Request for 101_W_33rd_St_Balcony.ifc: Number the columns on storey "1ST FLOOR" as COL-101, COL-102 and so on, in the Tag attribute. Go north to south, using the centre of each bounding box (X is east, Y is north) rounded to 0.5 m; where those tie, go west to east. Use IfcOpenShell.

First a look at what the model holds.

```python
import ifcopenshell
import ifcopenshell.util.element
import ifcopenshell.util.placement

model = ifcopenshell.open("101_W_33rd_St_Balcony.ifc")
print(model.schema)
storey = next(s for s in model.by_type("IfcBuildingStorey") if s.Name == "1ST FLOOR")
columns = [e for e in ifcopenshell.util.element.get_decomposition(storey) if e.is_a("IfcColumn")]
for e in sorted(columns, key=lambda e: e.id()):
    origin = ifcopenshell.util.placement.get_local_placement(e.ObjectPlacement)[:3, 3]
    print(e.id(), e.Tag, e.Name, origin.round(2) + 0.0, sep=" | ")
```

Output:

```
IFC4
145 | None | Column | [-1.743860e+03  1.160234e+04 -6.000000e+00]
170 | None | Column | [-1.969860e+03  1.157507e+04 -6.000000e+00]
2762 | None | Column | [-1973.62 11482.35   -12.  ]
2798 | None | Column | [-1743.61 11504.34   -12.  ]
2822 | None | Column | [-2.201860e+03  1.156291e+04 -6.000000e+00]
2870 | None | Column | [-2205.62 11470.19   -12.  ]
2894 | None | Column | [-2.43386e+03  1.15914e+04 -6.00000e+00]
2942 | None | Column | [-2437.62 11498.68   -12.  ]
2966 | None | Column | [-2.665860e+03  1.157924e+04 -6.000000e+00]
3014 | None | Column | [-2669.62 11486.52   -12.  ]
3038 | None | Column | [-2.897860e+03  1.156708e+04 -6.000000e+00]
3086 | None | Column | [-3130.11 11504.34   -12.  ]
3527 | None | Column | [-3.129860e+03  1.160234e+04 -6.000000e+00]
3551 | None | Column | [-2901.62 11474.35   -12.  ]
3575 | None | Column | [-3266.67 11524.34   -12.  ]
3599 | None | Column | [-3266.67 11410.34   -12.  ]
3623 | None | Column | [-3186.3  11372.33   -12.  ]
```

```python
import ifcopenshell
import ifcopenshell.geom
import ifcopenshell.util.element
import ifcopenshell.util.shape

model = ifcopenshell.open("101_W_33rd_St_Balcony.ifc")
settings = ifcopenshell.geom.settings()
settings.set("use-world-coords", True)


def centre(element):
    shape = ifcopenshell.geom.create_shape(settings, element)
    return ifcopenshell.util.shape.get_bbox_centroid(shape.geometry)


storey = next(s for s in model.by_type("IfcBuildingStorey") if s.Name == "1ST FLOOR")
columns = [e for e in ifcopenshell.util.element.get_decomposition(storey) if e.is_a("IfcColumn")]

# Insertion points can sit at a corner or the storey origin, so sort by the geometry (in metres).
centres = {e: centre(e) for e in columns}
columns.sort(key=lambda e: (-round(centres[e][1] / 0.5), centres[e][0]))

for i, e in enumerate(columns, start=1):
    number = f"COL-1{i:02d}"
    e.Tag = number
    print(e.id(), number)

model.write("101_W_33rd_St_Balcony-out.ifc")
```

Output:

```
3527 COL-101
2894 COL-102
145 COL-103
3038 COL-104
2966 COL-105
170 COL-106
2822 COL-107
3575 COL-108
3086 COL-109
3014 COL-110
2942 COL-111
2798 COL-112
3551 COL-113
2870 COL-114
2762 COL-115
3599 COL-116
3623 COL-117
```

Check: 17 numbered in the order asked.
